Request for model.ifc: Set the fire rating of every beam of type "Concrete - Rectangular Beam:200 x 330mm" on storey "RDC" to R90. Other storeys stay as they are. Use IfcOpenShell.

First a look at what the model holds.

```python
import ifcopenshell
import ifcopenshell.util.element

model = ifcopenshell.open("model.ifc")
print(model.schema)
storey = next(s for s in model.by_type("IfcBuildingStorey") if s.Name == "RDC")
beams = [e for e in ifcopenshell.util.element.get_decomposition(storey) if e.is_a("IfcBeam")]
seen = {}
for e in beams:
    element_type = ifcopenshell.util.element.get_type(e)
    key = (element_type.Name if element_type != e and element_type else None, ifcopenshell.util.element.get_pset(e, "Pset_BeamCommon", "FireRating"))
    seen[key] = seen.get(key, 0) + 1
for (name, value), count in sorted(seen.items(), key=str):
    print(count, "x", name, "|", value)
```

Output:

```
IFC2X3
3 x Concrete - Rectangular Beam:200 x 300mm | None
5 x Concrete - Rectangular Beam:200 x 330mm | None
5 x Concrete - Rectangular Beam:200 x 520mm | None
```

```python
import ifcopenshell
import ifcopenshell.api.pset
import ifcopenshell.util.element

model = ifcopenshell.open("model.ifc")

storey = next(s for s in model.by_type("IfcBuildingStorey") if s.Name == "RDC")
beams = [e for e in ifcopenshell.util.element.get_decomposition(storey) if e.is_a("IfcBeam")]

count = 0
for e in beams:
    element_type = ifcopenshell.util.element.get_type(e)
    if element_type in (None, e) or element_type.Name != "Concrete - Rectangular Beam:200 x 330mm":
        continue
    # add_pset returns the element's existing set when there is one.
    pset = ifcopenshell.api.pset.add_pset(model, product=e, name="Pset_BeamCommon")
    ifcopenshell.api.pset.edit_pset(model, pset=pset, properties={"FireRating": "R90"})
    count += 1

print(count, "beams updated")

model.write("model-out.ifc")
```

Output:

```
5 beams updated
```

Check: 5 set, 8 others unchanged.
